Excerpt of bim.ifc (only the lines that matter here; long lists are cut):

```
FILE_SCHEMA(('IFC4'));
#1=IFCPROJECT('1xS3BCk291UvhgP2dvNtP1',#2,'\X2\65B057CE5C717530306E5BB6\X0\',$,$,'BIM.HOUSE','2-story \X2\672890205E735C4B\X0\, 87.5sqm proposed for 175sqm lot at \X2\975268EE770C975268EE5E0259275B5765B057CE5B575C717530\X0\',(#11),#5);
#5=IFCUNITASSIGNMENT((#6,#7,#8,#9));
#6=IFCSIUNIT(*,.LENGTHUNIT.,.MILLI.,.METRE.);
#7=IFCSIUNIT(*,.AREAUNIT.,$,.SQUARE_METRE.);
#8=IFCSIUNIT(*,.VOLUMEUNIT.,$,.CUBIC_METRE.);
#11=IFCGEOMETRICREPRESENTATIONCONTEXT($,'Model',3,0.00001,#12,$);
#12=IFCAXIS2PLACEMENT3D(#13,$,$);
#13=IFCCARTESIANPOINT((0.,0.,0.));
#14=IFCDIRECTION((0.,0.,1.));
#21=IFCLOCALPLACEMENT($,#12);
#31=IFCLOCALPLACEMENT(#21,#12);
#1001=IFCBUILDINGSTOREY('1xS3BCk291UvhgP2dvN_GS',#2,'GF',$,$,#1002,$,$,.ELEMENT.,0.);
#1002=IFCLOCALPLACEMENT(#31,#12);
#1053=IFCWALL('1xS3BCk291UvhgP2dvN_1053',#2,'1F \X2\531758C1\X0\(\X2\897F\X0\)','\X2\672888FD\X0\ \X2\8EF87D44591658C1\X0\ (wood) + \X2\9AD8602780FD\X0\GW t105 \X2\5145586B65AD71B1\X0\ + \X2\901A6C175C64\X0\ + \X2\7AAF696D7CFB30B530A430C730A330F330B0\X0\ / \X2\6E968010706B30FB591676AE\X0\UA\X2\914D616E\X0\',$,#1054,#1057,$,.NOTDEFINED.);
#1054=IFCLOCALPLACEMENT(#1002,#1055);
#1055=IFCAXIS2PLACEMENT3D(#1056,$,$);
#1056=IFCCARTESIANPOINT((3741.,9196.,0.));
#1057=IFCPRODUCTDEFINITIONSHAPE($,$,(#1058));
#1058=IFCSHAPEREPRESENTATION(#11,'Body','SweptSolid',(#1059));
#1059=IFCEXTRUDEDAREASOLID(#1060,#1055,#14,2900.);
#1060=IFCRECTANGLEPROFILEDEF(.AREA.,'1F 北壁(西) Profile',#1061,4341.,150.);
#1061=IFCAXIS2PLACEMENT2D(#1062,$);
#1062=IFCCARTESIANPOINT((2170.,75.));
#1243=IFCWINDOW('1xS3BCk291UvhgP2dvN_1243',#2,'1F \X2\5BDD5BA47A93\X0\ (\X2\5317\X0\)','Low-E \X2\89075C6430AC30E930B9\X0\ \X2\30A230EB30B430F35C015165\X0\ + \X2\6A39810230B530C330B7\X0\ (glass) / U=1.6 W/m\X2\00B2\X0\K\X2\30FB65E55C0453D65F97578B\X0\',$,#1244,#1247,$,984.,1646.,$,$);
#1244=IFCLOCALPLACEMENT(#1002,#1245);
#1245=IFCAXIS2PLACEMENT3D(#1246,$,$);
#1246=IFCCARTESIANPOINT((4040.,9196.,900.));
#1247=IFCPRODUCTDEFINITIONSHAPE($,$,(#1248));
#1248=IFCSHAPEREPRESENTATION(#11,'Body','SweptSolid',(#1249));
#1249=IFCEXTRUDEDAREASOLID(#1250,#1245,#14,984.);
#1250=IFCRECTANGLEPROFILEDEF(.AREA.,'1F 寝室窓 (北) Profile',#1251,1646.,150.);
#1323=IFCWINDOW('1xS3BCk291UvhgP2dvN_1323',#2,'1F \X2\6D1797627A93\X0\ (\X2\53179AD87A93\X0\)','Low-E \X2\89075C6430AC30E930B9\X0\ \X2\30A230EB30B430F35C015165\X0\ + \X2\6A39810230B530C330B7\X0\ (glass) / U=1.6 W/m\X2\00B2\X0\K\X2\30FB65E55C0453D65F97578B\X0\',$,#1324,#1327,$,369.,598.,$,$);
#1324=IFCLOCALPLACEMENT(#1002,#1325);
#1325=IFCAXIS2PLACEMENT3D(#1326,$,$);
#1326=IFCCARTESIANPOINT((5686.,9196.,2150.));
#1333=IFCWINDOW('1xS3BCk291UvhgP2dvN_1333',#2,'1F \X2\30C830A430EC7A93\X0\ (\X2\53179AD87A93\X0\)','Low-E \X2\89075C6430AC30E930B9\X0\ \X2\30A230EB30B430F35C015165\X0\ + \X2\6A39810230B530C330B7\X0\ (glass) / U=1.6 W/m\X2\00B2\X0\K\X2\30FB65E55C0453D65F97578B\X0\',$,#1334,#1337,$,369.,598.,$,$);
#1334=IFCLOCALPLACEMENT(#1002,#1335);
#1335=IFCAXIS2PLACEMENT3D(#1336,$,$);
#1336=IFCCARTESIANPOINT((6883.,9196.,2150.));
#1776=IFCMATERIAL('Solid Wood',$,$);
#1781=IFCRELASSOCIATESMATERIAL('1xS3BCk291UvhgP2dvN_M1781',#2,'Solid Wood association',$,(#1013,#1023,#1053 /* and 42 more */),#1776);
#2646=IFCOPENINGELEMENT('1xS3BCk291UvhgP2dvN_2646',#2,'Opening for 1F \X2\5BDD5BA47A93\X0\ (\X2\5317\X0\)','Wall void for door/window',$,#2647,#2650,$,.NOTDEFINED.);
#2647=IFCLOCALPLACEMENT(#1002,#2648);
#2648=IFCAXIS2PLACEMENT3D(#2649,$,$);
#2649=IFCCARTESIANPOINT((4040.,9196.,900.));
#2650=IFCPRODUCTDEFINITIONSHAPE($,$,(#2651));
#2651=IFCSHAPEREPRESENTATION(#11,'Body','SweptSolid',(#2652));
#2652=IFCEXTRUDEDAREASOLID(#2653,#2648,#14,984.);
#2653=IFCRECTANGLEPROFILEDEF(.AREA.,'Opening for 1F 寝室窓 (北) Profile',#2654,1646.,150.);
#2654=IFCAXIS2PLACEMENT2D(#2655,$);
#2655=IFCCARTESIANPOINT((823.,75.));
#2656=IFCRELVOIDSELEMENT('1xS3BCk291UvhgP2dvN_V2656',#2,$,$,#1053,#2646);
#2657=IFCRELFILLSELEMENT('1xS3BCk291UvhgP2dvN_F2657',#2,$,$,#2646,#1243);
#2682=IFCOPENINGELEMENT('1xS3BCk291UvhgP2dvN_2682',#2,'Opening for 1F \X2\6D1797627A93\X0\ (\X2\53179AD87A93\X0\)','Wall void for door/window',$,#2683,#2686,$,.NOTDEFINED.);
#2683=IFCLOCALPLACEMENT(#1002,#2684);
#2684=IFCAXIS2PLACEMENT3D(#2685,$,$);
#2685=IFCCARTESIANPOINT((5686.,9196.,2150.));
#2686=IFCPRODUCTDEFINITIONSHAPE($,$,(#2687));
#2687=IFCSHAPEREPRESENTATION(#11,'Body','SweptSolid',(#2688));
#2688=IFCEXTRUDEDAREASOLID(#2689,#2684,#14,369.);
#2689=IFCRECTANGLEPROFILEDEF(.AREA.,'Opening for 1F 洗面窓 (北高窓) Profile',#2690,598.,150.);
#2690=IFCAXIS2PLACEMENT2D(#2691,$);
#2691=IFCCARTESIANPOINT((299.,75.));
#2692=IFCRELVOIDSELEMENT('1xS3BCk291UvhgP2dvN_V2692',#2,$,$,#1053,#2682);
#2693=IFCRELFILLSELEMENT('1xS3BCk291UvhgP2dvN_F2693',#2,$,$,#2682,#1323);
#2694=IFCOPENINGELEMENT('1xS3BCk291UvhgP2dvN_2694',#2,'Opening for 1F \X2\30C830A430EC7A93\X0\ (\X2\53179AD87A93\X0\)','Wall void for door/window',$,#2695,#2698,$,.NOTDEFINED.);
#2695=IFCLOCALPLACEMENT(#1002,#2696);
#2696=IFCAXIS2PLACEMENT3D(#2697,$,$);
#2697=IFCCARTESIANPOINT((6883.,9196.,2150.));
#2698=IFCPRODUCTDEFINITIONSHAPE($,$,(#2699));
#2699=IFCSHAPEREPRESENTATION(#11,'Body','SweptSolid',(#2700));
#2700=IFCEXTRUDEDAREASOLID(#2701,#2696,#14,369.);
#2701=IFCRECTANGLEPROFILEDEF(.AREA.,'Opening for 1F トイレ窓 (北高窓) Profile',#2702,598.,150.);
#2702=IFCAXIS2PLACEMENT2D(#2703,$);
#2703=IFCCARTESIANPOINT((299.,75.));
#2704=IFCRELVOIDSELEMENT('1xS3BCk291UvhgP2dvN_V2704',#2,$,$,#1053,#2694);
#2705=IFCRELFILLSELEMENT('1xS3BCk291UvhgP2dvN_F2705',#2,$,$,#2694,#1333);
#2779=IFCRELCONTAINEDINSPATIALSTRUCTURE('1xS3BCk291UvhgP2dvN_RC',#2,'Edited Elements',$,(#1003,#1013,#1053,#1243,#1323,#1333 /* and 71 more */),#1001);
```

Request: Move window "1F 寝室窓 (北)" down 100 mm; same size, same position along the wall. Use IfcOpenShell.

```python
import numpy as np
import ifcopenshell
import ifcopenshell.api.geometry
import ifcopenshell.util.placement
import ifcopenshell.util.unit

model = ifcopenshell.open("bim.ifc")
unit_scale = ifcopenshell.util.unit.calculate_unit_scale(model)

window = model.by_guid("1xS3BCk291UvhgP2dvN_1243")
opening = window.FillsVoids[0].RelatingOpeningElement
dz = -100.0

shift = np.array([0.0, 0.0, dz])
# The window is not placed relative to its opening, so move both.
for product in (opening, window):
    matrix = ifcopenshell.util.placement.get_local_placement(product.ObjectPlacement)
    matrix[:3, 3] += shift
    ifcopenshell.api.geometry.edit_object_placement(model, product=product, matrix=matrix, is_si=False)

print(f"moved by {dz * unit_scale:+.3f} m")

model.write("bim-out.ifc")
```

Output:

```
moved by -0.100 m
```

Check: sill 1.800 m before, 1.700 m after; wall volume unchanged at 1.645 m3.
